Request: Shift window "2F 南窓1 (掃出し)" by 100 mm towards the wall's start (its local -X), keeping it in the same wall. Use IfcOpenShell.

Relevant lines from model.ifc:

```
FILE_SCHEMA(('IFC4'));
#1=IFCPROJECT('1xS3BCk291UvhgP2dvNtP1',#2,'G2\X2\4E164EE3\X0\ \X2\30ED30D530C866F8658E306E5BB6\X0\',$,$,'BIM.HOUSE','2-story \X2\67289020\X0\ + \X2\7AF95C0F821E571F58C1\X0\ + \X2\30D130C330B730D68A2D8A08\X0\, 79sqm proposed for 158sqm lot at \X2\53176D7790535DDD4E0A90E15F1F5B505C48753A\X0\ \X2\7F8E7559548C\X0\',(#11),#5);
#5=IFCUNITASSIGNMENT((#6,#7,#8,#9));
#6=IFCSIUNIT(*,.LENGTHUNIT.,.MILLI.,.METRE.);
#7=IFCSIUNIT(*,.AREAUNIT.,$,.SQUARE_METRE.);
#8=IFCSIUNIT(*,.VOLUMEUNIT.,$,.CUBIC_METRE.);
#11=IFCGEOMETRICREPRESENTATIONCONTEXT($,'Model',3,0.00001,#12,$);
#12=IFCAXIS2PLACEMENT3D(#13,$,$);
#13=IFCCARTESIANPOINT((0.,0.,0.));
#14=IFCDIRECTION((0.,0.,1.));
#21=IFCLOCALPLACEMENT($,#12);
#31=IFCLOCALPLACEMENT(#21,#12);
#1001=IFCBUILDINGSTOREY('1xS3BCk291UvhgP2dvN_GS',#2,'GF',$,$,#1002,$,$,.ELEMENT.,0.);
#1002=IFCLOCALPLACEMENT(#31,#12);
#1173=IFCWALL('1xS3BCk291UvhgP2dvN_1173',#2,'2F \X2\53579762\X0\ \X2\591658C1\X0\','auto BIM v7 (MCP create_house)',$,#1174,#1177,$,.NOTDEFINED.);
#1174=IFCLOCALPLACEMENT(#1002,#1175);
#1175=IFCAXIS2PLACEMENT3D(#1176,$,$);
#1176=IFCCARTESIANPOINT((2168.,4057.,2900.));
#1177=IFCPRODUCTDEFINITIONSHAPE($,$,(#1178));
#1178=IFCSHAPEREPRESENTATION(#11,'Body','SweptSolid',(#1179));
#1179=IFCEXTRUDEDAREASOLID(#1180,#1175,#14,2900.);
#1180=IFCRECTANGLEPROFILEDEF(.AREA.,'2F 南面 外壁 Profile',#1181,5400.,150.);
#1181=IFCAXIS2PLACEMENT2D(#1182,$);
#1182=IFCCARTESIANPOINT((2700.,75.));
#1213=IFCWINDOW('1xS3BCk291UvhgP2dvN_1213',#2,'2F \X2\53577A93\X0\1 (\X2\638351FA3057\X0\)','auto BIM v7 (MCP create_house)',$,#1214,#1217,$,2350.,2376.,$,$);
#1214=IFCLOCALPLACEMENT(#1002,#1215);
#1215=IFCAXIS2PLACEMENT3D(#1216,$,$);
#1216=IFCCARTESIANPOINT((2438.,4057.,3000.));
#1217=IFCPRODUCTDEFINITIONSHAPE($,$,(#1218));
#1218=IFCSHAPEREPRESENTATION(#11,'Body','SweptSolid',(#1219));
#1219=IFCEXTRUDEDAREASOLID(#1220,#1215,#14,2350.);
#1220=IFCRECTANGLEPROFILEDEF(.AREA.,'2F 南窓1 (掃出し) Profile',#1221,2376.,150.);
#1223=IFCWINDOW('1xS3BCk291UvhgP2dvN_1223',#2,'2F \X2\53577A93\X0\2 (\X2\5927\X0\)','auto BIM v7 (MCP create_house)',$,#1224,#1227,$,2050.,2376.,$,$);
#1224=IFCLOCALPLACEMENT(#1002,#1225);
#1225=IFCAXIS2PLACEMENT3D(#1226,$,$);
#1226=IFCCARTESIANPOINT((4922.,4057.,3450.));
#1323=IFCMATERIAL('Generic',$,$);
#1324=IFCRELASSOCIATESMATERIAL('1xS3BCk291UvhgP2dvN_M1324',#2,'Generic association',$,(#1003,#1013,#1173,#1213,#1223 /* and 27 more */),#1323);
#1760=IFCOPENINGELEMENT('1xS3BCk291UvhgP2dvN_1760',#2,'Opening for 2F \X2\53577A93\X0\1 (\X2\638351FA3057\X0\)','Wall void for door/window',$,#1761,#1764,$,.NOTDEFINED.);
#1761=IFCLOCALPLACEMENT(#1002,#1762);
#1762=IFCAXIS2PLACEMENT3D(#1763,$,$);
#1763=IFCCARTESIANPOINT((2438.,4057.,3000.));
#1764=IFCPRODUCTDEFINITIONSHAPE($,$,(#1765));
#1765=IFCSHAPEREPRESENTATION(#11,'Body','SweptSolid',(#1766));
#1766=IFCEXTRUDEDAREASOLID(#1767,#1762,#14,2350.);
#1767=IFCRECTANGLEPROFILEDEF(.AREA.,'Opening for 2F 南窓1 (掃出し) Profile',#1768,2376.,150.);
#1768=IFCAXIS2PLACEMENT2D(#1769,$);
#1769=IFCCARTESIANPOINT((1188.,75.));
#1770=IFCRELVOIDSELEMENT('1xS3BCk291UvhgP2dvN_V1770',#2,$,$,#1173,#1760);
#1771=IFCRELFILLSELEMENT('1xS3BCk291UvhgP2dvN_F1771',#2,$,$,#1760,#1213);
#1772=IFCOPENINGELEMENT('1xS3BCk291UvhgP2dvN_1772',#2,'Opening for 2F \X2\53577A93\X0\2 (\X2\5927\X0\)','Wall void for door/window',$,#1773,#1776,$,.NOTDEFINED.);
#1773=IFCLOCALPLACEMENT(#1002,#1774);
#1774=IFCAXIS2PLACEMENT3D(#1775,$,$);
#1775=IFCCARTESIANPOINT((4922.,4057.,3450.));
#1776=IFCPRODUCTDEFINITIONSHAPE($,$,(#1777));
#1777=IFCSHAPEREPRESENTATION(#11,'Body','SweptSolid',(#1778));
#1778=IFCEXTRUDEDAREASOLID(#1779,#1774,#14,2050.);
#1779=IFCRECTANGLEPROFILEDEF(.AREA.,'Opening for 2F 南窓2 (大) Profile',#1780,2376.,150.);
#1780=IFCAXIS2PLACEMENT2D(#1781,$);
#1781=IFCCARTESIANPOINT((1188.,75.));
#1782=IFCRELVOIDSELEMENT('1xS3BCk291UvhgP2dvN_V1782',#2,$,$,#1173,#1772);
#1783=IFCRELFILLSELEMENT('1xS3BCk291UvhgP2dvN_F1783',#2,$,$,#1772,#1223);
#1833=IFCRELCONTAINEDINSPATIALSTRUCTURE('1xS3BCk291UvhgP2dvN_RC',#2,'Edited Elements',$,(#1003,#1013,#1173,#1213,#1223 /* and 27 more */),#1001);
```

```python
import ifcopenshell
import ifcopenshell.api.geometry
import ifcopenshell.util.placement

model = ifcopenshell.open("model.ifc")

window = model.by_guid("1xS3BCk291UvhgP2dvN_1213")
opening = window.FillsVoids[0].RelatingOpeningElement
wall = opening.VoidsElements[0].RelatingBuildingElement

wall_matrix = ifcopenshell.util.placement.get_local_placement(wall.ObjectPlacement)
shift = wall_matrix[:3, 0] * -100.0
before = ifcopenshell.util.placement.get_local_placement(window.ObjectPlacement)[:3, 3].copy()

# The window is not placed relative to its opening, so move both.
for product in (opening, window):
    matrix = ifcopenshell.util.placement.get_local_placement(product.ObjectPlacement)
    matrix[:3, 3] += shift
    ifcopenshell.api.geometry.edit_object_placement(model, product=product, matrix=matrix, is_si=False)

after = ifcopenshell.util.placement.get_local_placement(window.ObjectPlacement)[:3, 3]
print("window moved by", (after - before).round(3) + 0.0)

model.write("model_updated.ifc")
```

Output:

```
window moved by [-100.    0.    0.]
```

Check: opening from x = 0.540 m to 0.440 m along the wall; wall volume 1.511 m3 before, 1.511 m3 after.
